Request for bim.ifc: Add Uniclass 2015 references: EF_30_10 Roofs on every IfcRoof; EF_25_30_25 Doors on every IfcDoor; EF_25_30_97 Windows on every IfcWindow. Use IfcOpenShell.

First a look at what the model holds.

```python
import ifcopenshell

model = ifcopenshell.open("bim.ifc")
print(model.schema)
print("classifications:", [c.Name for c in model.by_type("IfcClassification")])
for ifc_class in ("IfcDoor", "IfcRoof", "IfcStair", "IfcWall", "IfcWindow"):
    print(ifc_class, len(model.by_type(ifc_class)))
```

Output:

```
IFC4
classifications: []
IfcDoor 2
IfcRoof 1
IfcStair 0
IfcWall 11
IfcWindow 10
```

```python
import ifcopenshell
import ifcopenshell.api.classification

model = ifcopenshell.open("bim.ifc")

system = ifcopenshell.api.classification.add_classification(model, classification="Uniclass 2015")

codes = {
    "IfcRoof": ("EF_30_10", "Roofs"),
    "IfcDoor": ("EF_25_30_25", "Doors"),
    "IfcWindow": ("EF_25_30_97", "Windows"),
}
for ifc_class, (code, name) in codes.items():
    products = model.by_type(ifc_class)
    ifcopenshell.api.classification.add_reference(
        model, products=products, classification=system, identification=code, name=name
    )
    print(code, len(products))

model.write("bim_rev.ifc")
```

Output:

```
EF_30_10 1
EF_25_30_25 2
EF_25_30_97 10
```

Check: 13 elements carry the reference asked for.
